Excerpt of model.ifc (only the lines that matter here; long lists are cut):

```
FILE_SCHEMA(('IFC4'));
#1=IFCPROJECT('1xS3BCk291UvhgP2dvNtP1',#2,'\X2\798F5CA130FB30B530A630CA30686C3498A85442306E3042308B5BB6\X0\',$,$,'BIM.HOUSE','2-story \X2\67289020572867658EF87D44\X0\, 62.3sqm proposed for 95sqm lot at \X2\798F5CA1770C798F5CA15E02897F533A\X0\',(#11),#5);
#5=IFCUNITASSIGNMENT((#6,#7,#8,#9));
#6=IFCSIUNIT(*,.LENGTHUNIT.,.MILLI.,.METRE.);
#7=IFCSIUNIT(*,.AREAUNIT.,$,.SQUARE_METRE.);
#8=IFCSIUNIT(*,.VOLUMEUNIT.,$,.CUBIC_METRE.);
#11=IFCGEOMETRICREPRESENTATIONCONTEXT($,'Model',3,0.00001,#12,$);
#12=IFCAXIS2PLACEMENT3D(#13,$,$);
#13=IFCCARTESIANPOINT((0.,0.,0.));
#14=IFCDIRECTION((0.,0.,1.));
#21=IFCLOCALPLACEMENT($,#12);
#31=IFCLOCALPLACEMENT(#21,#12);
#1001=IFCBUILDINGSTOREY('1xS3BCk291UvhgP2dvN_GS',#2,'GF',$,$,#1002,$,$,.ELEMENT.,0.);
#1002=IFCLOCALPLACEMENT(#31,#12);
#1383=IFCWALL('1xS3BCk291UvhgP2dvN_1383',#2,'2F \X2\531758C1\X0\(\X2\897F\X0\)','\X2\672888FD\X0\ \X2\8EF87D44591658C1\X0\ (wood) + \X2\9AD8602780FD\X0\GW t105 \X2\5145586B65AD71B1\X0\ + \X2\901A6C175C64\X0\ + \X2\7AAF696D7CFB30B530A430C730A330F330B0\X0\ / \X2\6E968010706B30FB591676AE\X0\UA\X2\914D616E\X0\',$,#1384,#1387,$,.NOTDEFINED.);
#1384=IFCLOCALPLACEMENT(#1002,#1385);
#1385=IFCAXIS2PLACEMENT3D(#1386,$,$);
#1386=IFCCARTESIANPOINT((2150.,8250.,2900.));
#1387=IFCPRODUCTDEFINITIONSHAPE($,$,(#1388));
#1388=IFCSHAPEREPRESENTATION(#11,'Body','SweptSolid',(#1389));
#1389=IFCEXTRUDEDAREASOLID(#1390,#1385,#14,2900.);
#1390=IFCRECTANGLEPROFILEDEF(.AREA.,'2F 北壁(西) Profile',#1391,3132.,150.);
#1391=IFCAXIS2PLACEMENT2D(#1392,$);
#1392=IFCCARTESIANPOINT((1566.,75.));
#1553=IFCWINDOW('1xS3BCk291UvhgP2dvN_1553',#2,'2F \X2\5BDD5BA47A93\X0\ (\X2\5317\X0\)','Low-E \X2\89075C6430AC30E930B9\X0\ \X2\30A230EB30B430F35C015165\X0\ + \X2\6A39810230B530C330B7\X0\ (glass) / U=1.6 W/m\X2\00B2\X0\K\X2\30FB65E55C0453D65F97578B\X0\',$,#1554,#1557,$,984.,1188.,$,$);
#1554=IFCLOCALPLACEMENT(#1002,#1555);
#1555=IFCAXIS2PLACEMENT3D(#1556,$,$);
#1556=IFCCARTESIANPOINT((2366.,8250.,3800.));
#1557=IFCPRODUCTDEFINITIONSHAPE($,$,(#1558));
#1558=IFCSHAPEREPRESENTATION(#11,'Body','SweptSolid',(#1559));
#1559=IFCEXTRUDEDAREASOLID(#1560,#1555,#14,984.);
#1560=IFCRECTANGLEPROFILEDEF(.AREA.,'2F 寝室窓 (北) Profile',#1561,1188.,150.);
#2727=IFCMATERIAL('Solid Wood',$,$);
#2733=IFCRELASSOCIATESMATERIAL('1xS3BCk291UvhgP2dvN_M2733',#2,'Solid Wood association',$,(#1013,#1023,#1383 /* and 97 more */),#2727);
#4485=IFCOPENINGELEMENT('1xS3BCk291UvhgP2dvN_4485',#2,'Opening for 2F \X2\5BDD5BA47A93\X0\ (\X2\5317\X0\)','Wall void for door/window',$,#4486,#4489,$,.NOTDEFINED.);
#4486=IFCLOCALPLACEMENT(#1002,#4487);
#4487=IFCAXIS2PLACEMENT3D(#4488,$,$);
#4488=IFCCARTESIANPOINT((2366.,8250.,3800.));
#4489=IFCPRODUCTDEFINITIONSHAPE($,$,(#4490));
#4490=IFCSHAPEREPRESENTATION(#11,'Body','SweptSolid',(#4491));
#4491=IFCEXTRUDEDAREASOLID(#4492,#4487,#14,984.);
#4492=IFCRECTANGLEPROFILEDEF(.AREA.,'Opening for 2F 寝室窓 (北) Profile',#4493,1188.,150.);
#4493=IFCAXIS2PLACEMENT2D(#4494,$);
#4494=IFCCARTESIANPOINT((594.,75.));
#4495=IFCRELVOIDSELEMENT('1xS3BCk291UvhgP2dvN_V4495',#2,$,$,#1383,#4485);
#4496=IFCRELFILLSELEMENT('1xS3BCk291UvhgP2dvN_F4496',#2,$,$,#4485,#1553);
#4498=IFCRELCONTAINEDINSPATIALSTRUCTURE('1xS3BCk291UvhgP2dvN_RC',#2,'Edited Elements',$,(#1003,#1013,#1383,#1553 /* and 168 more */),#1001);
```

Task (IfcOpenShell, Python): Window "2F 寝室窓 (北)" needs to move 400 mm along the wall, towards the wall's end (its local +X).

```python
import ifcopenshell
import ifcopenshell.api.geometry
import ifcopenshell.util.placement
import ifcopenshell.util.unit

model = ifcopenshell.open("model.ifc")
unit_scale = ifcopenshell.util.unit.calculate_unit_scale(model)

window = model.by_guid("1xS3BCk291UvhgP2dvN_1553")
opening = window.FillsVoids[0].RelatingOpeningElement
wall = opening.VoidsElements[0].RelatingBuildingElement

wall_matrix = ifcopenshell.util.placement.get_local_placement(wall.ObjectPlacement)
shift = wall_matrix[:3, 0] * 0.4 / unit_scale
before = ifcopenshell.util.placement.get_local_placement(window.ObjectPlacement)[:3, 3].copy()

# The window is not placed relative to its opening, so move both.
for product in (opening, window):
    matrix = ifcopenshell.util.placement.get_local_placement(product.ObjectPlacement)
    matrix[:3, 3] += shift
    ifcopenshell.api.geometry.edit_object_placement(model, product=product, matrix=matrix, is_si=False)

after = ifcopenshell.util.placement.get_local_placement(window.ObjectPlacement)[:3, 3]
print("window moved by", (after - before).round(3) + 0.0)

model.write("model_edited.ifc")
```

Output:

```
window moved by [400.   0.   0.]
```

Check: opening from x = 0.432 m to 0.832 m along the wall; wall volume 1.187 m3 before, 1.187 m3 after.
